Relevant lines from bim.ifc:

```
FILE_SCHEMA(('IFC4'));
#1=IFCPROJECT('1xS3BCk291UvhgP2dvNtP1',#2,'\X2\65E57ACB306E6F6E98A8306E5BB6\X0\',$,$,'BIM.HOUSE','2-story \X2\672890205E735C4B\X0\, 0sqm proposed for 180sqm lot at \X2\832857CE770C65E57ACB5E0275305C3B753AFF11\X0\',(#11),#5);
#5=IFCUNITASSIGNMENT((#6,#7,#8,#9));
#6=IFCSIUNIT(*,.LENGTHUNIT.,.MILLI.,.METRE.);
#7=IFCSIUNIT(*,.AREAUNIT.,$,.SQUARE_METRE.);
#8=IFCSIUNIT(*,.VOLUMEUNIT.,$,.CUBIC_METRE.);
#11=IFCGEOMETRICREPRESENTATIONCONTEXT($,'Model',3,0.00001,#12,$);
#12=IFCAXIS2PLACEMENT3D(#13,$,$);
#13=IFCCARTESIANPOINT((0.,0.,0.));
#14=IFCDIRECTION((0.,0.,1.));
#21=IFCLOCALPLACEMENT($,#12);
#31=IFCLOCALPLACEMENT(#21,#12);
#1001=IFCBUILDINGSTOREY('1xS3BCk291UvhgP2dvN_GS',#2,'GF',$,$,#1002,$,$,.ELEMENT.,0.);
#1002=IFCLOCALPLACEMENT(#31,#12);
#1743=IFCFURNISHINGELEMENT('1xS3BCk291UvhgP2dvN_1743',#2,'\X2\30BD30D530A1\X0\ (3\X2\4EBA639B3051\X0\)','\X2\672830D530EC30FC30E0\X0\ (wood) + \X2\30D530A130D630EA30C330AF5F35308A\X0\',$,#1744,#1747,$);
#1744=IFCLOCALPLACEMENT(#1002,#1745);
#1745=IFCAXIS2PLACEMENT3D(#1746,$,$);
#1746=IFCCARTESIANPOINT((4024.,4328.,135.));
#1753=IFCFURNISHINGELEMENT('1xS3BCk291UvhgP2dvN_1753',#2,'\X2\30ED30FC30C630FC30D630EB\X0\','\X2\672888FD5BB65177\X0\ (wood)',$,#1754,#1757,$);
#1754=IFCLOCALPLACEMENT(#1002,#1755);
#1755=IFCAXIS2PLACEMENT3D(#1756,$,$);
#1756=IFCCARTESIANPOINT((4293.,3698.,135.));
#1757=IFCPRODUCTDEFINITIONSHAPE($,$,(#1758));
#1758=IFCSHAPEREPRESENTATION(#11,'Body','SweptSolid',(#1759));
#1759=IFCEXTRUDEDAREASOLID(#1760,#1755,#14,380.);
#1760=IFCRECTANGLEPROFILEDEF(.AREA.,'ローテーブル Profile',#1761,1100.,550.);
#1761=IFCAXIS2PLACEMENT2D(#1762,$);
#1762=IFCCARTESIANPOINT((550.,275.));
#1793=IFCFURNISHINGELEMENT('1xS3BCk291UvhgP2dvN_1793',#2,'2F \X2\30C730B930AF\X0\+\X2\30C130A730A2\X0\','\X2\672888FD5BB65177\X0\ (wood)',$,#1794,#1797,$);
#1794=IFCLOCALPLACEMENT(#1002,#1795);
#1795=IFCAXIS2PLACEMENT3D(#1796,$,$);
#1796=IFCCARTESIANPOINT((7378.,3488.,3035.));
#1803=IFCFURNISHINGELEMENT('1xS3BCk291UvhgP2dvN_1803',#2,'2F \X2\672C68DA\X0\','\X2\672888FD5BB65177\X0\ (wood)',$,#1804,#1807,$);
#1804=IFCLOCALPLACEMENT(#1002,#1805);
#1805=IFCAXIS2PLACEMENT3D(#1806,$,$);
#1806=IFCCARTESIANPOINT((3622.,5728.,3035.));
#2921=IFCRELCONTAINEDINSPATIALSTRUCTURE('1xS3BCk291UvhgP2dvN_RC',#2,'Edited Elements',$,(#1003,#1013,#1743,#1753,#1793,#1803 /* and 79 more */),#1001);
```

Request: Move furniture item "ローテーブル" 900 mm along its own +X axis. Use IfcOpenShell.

```python
import ifcopenshell
import ifcopenshell.api.geometry
import ifcopenshell.util.placement

model = ifcopenshell.open("bim.ifc")

item = model.by_guid("1xS3BCk291UvhgP2dvN_1753")
matrix = ifcopenshell.util.placement.get_local_placement(item.ObjectPlacement)
matrix[:3, 3] += matrix[:3, 0] * 900.0
ifcopenshell.api.geometry.edit_object_placement(model, product=item, matrix=matrix, is_si=False)

print(ifcopenshell.util.placement.get_local_placement(item.ObjectPlacement).round(3) + 0.0)

model.write("bim_updated.ifc")
```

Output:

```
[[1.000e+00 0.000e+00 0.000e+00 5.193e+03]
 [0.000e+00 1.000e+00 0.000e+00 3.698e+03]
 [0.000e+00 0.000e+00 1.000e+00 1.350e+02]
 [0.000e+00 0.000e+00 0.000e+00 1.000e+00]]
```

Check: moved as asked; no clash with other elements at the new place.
